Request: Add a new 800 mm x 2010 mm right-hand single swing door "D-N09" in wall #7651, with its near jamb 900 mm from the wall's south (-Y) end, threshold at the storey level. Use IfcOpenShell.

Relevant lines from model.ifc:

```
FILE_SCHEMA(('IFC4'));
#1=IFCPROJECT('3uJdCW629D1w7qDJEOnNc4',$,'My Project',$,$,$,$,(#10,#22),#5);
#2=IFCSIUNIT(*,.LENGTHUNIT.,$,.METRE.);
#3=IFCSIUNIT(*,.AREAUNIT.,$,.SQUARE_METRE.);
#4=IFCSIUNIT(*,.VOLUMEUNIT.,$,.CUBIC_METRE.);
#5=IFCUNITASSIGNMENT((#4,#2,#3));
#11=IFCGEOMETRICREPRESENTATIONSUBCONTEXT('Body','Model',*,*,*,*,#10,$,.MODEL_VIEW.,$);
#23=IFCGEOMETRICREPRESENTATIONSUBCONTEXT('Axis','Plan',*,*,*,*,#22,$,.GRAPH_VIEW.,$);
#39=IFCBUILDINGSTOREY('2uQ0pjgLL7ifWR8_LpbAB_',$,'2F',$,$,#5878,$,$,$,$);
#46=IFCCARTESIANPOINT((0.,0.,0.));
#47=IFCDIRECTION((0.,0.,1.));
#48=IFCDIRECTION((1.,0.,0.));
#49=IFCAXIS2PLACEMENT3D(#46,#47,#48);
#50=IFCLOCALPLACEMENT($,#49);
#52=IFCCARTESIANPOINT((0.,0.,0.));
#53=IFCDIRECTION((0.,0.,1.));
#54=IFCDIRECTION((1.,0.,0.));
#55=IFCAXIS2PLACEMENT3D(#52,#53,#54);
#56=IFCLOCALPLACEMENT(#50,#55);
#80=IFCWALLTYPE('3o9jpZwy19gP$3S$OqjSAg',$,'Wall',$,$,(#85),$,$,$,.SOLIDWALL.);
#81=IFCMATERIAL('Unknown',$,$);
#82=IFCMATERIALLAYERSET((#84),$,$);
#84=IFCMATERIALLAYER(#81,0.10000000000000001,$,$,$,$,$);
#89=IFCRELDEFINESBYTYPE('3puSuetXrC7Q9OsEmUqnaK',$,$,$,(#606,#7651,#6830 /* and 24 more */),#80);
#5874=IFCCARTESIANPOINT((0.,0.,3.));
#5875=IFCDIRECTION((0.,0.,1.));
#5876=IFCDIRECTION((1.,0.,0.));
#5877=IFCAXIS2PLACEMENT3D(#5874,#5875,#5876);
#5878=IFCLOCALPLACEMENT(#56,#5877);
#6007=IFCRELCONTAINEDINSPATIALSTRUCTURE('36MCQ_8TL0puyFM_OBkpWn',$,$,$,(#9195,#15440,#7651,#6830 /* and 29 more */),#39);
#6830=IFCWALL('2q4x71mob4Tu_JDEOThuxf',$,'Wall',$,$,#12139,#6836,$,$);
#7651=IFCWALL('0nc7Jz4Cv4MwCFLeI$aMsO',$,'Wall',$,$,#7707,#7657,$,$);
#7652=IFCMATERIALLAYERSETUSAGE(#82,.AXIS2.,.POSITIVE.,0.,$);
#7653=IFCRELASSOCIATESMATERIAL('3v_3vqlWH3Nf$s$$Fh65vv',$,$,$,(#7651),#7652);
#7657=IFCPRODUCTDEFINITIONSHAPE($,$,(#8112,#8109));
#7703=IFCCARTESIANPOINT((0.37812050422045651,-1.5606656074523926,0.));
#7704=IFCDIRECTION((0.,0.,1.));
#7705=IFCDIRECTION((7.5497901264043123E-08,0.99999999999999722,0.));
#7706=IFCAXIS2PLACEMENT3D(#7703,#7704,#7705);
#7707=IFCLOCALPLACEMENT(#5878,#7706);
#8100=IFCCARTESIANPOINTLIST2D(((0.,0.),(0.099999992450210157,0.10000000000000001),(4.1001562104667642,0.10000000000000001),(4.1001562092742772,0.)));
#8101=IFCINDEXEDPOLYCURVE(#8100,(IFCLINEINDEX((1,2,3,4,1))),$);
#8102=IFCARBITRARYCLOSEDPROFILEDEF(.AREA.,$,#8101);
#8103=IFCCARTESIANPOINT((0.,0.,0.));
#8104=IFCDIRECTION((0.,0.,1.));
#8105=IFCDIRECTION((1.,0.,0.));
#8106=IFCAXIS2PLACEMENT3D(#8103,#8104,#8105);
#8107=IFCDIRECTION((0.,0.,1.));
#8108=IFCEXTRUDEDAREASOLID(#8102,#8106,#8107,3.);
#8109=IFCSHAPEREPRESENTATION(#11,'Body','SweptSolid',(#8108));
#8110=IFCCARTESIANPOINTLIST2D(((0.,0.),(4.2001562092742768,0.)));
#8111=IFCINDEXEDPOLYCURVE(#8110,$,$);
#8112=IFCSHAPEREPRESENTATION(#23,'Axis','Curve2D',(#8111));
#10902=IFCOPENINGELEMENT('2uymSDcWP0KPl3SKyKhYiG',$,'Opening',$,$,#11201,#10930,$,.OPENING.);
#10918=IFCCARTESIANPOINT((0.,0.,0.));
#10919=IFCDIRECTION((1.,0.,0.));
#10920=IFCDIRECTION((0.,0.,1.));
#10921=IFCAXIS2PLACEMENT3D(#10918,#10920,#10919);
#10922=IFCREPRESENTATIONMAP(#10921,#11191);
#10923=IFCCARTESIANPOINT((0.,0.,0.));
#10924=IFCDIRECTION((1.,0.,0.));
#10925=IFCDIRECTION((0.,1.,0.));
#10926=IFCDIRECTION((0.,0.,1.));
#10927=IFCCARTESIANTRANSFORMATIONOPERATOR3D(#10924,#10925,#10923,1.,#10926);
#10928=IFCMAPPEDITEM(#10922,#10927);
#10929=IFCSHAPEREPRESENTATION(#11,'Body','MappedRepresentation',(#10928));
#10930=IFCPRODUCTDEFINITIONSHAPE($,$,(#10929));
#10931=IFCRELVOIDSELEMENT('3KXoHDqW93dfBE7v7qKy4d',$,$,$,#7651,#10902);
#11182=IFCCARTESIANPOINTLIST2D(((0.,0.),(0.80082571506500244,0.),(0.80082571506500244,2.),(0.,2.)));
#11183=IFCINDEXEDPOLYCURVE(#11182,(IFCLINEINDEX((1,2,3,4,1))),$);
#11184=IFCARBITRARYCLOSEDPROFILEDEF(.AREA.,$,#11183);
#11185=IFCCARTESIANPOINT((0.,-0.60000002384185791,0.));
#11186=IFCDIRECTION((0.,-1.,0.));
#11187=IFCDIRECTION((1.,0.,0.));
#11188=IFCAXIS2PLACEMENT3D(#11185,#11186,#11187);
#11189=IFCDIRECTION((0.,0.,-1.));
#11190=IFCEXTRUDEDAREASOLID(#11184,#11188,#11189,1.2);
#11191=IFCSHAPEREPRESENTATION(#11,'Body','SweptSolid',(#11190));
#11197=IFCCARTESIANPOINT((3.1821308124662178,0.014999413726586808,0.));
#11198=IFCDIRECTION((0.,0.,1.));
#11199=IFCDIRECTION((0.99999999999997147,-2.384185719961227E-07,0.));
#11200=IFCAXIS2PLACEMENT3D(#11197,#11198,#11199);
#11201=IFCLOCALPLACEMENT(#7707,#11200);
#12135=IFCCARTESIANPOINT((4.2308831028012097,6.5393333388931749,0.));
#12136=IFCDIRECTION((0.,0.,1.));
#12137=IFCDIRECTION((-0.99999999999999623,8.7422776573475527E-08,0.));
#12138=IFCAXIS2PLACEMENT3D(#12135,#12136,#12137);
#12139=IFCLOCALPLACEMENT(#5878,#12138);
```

```python
import numpy as np
import ifcopenshell
import ifcopenshell.api.feature
import ifcopenshell.api.geometry
import ifcopenshell.api.root
import ifcopenshell.api.spatial
import ifcopenshell.geom
import ifcopenshell.util.element
import ifcopenshell.util.placement
import ifcopenshell.util.representation
import ifcopenshell.util.shape
import ifcopenshell.util.unit

model = ifcopenshell.open("model.ifc")
unit_scale = ifcopenshell.util.unit.calculate_unit_scale(model)
settings = ifcopenshell.geom.settings()


def volume(element):
    """Net volume in cubic metres, openings subtracted."""
    shape = ifcopenshell.geom.create_shape(settings, element)
    return ifcopenshell.util.shape.get_volume(shape.geometry)


wall = model.by_id(7651)
storey = ifcopenshell.util.element.get_container(wall, ifc_class="IfcBuildingStorey")
context = ifcopenshell.util.representation.get_context(model, "Model", "Body", "MODEL_VIEW")
before = volume(wall)

width, height, from_end, sill = 0.8, 2.01, 0.9, 0.0  # metres

# The wall runs along its own X axis, and the end named is its -X end.
wall_shape = ifcopenshell.geom.create_shape(settings, wall)
x, y, z = ifcopenshell.util.shape.get_vertices(wall_shape.geometry).T
start = x.min() + from_end
face, thickness = float(y.min()), float(y.max() - y.min())
wall_matrix = ifcopenshell.util.placement.get_local_placement(wall.ObjectPlacement)
level = ifcopenshell.util.placement.get_local_placement(storey.ObjectPlacement)[2, 3]


def in_wall(x, y):
    """Placement at x, y metres in the wall's axes, at sill height."""
    matrix = wall_matrix.copy()
    matrix[:, 3] = wall_matrix @ np.array([x / unit_scale, y / unit_scale, 0.0, 1.0])
    matrix[2, 3] = level + sill / unit_scale
    return matrix


# Opening: a box that overshoots both wall faces by 50 mm.
opening = ifcopenshell.api.root.create_entity(model, ifc_class="IfcOpeningElement", predefined_type="OPENING")
box = ifcopenshell.api.geometry.add_wall_representation(
    model, context=context, length=width, height=height, thickness=thickness + 0.1
)
ifcopenshell.api.geometry.assign_representation(model, product=opening, representation=box)
ifcopenshell.api.geometry.edit_object_placement(model, product=opening, matrix=in_wall(start, face - 0.05), is_si=False)
ifcopenshell.api.feature.add_feature(model, feature=opening, element=wall)

door = ifcopenshell.api.root.create_entity(model, ifc_class="IfcDoor", name="D-N09", predefined_type="DOOR")
door.OverallWidth, door.OverallHeight = width / unit_scale, height / unit_scale
door.OperationType = "SINGLE_SWING_RIGHT"
body = ifcopenshell.api.geometry.add_door_representation(
    model,
    context=context,
    overall_width=door.OverallWidth,
    overall_height=door.OverallHeight,
    operation_type="SINGLE_SWING_RIGHT",
    lining_properties={"LiningDepth": thickness / unit_scale, "ThresholdDepth": thickness / unit_scale},
)
ifcopenshell.api.geometry.assign_representation(model, product=door, representation=body)
ifcopenshell.api.spatial.assign_container(model, products=[door], relating_structure=storey)
ifcopenshell.api.feature.add_filling(model, opening=opening, element=door)

# The lining spans the wall, so the door starts at the wall face.
ifcopenshell.api.geometry.edit_object_placement(model, product=door, matrix=in_wall(start, face), is_si=False)

after = volume(wall)

print(f"wall volume {before:.3f} -> {after:.3f} m3")

model.write("model_rev.ifc")
```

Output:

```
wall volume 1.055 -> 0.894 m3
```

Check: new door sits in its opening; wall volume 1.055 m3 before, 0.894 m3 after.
